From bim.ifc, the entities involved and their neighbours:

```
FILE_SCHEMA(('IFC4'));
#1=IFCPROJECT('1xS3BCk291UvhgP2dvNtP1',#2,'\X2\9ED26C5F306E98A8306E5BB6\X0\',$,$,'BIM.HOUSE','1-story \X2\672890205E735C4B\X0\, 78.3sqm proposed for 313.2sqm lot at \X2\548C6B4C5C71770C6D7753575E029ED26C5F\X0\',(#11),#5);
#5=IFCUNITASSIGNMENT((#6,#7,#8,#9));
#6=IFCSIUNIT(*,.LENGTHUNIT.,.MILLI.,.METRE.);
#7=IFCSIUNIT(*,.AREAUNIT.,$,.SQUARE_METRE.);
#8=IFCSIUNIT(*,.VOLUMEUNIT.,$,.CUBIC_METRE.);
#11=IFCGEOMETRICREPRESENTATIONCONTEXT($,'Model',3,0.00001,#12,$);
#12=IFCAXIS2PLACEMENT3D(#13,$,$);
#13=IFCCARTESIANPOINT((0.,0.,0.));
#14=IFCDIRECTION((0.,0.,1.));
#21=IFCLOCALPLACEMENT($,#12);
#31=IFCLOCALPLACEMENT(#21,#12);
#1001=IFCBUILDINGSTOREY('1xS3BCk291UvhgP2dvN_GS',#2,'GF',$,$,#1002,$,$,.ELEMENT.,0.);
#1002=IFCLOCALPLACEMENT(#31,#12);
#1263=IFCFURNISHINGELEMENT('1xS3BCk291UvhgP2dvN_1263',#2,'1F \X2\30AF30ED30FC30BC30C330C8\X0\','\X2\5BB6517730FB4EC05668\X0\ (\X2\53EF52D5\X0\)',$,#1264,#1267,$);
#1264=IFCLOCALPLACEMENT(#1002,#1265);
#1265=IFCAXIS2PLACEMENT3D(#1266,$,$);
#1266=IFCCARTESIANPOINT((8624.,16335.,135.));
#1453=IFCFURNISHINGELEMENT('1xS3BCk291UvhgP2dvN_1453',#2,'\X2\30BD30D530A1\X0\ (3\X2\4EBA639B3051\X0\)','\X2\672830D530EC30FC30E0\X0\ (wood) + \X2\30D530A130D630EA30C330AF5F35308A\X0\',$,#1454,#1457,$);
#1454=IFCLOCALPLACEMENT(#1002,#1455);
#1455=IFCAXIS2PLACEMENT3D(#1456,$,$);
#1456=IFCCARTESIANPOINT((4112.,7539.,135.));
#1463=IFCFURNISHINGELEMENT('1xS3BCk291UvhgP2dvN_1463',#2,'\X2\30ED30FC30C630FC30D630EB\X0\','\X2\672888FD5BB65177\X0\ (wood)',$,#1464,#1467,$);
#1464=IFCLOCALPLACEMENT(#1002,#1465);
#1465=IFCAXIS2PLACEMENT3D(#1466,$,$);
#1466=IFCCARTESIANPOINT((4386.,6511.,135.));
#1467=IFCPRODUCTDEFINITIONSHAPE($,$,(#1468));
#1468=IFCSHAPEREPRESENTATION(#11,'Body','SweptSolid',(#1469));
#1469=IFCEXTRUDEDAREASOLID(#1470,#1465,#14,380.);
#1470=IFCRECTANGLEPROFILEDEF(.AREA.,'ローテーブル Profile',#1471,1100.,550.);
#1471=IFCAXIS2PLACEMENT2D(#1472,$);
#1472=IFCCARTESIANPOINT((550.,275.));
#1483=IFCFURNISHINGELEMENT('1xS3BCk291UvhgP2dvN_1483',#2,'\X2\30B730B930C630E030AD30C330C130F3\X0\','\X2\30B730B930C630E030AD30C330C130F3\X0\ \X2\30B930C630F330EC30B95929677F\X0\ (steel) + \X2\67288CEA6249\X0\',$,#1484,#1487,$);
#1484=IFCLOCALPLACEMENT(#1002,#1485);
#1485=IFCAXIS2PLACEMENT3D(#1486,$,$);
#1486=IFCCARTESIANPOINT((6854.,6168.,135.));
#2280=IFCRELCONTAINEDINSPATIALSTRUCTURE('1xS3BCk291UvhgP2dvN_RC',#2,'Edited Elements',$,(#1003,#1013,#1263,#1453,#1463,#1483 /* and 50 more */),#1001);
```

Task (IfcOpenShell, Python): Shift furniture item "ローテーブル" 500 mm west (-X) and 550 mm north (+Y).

```python
import ifcopenshell
import ifcopenshell.api.geometry
import ifcopenshell.util.placement

model = ifcopenshell.open("bim.ifc")

item = model.by_guid("1xS3BCk291UvhgP2dvN_1463")
matrix = ifcopenshell.util.placement.get_local_placement(item.ObjectPlacement)
matrix[0, 3] -= 500.0
matrix[1, 3] += 550.0
ifcopenshell.api.geometry.edit_object_placement(model, product=item, matrix=matrix, is_si=False)

print(ifcopenshell.util.placement.get_local_placement(item.ObjectPlacement).round(3) + 0.0)

model.write("bim_v2.ifc")
```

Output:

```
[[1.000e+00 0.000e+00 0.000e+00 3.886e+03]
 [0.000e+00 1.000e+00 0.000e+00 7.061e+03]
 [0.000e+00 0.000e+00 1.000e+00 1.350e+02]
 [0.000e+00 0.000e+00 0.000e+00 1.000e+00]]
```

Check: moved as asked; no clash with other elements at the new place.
